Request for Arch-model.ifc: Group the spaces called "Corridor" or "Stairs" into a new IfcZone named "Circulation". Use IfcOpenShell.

First a look at what the model holds.

```python
import ifcopenshell

model = ifcopenshell.open("Arch-model.ifc")
print(model.schema)
seen = {}
for space in model.by_type("IfcSpace"):
    seen[space.LongName] = seen.get(space.LongName, 0) + 1
for name, count in sorted(seen.items(), key=str):
    print(count, "x", name)
print("zones:", [z.Name for z in model.by_type("IfcZone")][:20])
```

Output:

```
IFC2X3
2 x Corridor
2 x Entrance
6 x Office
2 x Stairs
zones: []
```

```python
import ifcopenshell
import ifcopenshell.api.group
import ifcopenshell.api.root

model = ifcopenshell.open("Arch-model.ifc")

names = {"Corridor", "Stairs"}
spaces = [s for s in model.by_type("IfcSpace") if s.LongName in names]

zone = ifcopenshell.api.root.create_entity(model, ifc_class="IfcZone", name="Circulation")
ifcopenshell.api.group.assign_group(model, products=spaces, group=zone)
print(len(spaces), "spaces in", zone.Name)

model.write("Arch-model-out.ifc")
```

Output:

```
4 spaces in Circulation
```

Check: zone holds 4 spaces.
